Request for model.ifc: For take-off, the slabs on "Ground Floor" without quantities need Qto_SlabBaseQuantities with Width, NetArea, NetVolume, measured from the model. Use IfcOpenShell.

First a look at what the model holds.

```python
import ifcopenshell
import ifcopenshell.util.element
import ifcopenshell.util.unit

model = ifcopenshell.open("model.ifc")
print(model.schema)
for unit_type in ("LENGTHUNIT", "AREAUNIT", "VOLUMEUNIT"):
    print(unit_type, ifcopenshell.util.unit.calculate_unit_scale(model, unit_type))
storey = next(s for s in model.by_type("IfcBuildingStorey") if s.Name == "Ground Floor")
slabs = [e for e in ifcopenshell.util.element.get_decomposition(storey) if e.is_a("IfcSlab")]
for e in sorted(slabs, key=lambda e: e.id()):
    print(e.id(), e.is_a(), e.Name, list(ifcopenshell.util.element.get_psets(e, qtos_only=True)), sep=" | ")
```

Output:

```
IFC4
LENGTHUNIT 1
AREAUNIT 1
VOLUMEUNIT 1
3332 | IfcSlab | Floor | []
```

```python
import ifcopenshell
import ifcopenshell.api.pset
import ifcopenshell.geom
import ifcopenshell.util.element
import ifcopenshell.util.shape
import ifcopenshell.util.unit

model = ifcopenshell.open("model.ifc")
unit_scale = ifcopenshell.util.unit.calculate_unit_scale(model)
area_scale = ifcopenshell.util.unit.calculate_unit_scale(model, "AREAUNIT")
volume_scale = ifcopenshell.util.unit.calculate_unit_scale(model, "VOLUMEUNIT")
settings = ifcopenshell.geom.settings()

storey = next(s for s in model.by_type("IfcBuildingStorey") if s.Name == "Ground Floor")
slabs = [e for e in ifcopenshell.util.element.get_decomposition(storey) if e.is_a("IfcSlab")]

for e in sorted(slabs, key=lambda e: e.id()):
    if ifcopenshell.util.element.get_psets(e, qtos_only=True, should_inherit=False):
        continue
    # Geometry comes back in metres, in the element's own axes.
    shape = ifcopenshell.geom.create_shape(settings, e)
    values = {
        "Width": ifcopenshell.util.shape.get_z(shape.geometry) / unit_scale,
        "NetArea": ifcopenshell.util.shape.get_footprint_area(shape.geometry) / area_scale,
        "NetVolume": ifcopenshell.util.shape.get_volume(shape.geometry) / volume_scale,
    }
    qto = ifcopenshell.api.pset.add_qto(model, product=e, name="Qto_SlabBaseQuantities")
    ifcopenshell.api.pset.edit_qto(model, qto=qto, properties=values)
    print(e.id(), {k: round(v, 3) for k, v in values.items()})

model.write("model_updated.ifc")
```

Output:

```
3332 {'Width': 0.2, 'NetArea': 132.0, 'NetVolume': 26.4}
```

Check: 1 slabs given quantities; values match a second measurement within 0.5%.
